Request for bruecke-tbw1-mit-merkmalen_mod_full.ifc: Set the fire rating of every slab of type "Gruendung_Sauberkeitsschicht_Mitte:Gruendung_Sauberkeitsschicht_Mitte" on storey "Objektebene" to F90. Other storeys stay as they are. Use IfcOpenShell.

First a look at what the model holds.

```python
import ifcopenshell
import ifcopenshell.util.element

model = ifcopenshell.open("bruecke-tbw1-mit-merkmalen_mod_full.ifc")
print(model.schema)
storey = next(s for s in model.by_type("IfcBuildingStorey") if s.Name == "Objektebene")
slabs = [e for e in ifcopenshell.util.element.get_decomposition(storey) if e.is_a("IfcSlab")]
seen = {}
for e in slabs:
    element_type = ifcopenshell.util.element.get_type(e)
    key = (element_type.Name if element_type != e and element_type else None, ifcopenshell.util.element.get_pset(e, "Pset_SlabCommon", "FireRating"))
    seen[key] = seen.get(key, 0) + 1
for (name, value), count in sorted(seen.items(), key=str):
    print(count, "x", name, "|", value)
```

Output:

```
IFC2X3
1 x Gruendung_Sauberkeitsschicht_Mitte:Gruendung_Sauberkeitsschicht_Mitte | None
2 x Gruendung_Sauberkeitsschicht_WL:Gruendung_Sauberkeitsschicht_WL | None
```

```python
import ifcopenshell
import ifcopenshell.api.pset
import ifcopenshell.util.element

model = ifcopenshell.open("bruecke-tbw1-mit-merkmalen_mod_full.ifc")

storey = next(s for s in model.by_type("IfcBuildingStorey") if s.Name == "Objektebene")
slabs = [e for e in ifcopenshell.util.element.get_decomposition(storey) if e.is_a("IfcSlab")]

count = 0
for e in slabs:
    element_type = ifcopenshell.util.element.get_type(e)
    if element_type in (None, e) or element_type.Name != "Gruendung_Sauberkeitsschicht_Mitte:Gruendung_Sauberkeitsschicht_Mitte":
        continue
    # add_pset returns the element's existing set when there is one.
    pset = ifcopenshell.api.pset.add_pset(model, product=e, name="Pset_SlabCommon")
    ifcopenshell.api.pset.edit_pset(model, pset=pset, properties={"FireRating": "F90"})
    count += 1

print(count, "slabs updated")

model.write("bruecke-tbw1-mit-merkmalen_mod_full-out.ifc")
```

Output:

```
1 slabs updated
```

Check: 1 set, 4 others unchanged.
